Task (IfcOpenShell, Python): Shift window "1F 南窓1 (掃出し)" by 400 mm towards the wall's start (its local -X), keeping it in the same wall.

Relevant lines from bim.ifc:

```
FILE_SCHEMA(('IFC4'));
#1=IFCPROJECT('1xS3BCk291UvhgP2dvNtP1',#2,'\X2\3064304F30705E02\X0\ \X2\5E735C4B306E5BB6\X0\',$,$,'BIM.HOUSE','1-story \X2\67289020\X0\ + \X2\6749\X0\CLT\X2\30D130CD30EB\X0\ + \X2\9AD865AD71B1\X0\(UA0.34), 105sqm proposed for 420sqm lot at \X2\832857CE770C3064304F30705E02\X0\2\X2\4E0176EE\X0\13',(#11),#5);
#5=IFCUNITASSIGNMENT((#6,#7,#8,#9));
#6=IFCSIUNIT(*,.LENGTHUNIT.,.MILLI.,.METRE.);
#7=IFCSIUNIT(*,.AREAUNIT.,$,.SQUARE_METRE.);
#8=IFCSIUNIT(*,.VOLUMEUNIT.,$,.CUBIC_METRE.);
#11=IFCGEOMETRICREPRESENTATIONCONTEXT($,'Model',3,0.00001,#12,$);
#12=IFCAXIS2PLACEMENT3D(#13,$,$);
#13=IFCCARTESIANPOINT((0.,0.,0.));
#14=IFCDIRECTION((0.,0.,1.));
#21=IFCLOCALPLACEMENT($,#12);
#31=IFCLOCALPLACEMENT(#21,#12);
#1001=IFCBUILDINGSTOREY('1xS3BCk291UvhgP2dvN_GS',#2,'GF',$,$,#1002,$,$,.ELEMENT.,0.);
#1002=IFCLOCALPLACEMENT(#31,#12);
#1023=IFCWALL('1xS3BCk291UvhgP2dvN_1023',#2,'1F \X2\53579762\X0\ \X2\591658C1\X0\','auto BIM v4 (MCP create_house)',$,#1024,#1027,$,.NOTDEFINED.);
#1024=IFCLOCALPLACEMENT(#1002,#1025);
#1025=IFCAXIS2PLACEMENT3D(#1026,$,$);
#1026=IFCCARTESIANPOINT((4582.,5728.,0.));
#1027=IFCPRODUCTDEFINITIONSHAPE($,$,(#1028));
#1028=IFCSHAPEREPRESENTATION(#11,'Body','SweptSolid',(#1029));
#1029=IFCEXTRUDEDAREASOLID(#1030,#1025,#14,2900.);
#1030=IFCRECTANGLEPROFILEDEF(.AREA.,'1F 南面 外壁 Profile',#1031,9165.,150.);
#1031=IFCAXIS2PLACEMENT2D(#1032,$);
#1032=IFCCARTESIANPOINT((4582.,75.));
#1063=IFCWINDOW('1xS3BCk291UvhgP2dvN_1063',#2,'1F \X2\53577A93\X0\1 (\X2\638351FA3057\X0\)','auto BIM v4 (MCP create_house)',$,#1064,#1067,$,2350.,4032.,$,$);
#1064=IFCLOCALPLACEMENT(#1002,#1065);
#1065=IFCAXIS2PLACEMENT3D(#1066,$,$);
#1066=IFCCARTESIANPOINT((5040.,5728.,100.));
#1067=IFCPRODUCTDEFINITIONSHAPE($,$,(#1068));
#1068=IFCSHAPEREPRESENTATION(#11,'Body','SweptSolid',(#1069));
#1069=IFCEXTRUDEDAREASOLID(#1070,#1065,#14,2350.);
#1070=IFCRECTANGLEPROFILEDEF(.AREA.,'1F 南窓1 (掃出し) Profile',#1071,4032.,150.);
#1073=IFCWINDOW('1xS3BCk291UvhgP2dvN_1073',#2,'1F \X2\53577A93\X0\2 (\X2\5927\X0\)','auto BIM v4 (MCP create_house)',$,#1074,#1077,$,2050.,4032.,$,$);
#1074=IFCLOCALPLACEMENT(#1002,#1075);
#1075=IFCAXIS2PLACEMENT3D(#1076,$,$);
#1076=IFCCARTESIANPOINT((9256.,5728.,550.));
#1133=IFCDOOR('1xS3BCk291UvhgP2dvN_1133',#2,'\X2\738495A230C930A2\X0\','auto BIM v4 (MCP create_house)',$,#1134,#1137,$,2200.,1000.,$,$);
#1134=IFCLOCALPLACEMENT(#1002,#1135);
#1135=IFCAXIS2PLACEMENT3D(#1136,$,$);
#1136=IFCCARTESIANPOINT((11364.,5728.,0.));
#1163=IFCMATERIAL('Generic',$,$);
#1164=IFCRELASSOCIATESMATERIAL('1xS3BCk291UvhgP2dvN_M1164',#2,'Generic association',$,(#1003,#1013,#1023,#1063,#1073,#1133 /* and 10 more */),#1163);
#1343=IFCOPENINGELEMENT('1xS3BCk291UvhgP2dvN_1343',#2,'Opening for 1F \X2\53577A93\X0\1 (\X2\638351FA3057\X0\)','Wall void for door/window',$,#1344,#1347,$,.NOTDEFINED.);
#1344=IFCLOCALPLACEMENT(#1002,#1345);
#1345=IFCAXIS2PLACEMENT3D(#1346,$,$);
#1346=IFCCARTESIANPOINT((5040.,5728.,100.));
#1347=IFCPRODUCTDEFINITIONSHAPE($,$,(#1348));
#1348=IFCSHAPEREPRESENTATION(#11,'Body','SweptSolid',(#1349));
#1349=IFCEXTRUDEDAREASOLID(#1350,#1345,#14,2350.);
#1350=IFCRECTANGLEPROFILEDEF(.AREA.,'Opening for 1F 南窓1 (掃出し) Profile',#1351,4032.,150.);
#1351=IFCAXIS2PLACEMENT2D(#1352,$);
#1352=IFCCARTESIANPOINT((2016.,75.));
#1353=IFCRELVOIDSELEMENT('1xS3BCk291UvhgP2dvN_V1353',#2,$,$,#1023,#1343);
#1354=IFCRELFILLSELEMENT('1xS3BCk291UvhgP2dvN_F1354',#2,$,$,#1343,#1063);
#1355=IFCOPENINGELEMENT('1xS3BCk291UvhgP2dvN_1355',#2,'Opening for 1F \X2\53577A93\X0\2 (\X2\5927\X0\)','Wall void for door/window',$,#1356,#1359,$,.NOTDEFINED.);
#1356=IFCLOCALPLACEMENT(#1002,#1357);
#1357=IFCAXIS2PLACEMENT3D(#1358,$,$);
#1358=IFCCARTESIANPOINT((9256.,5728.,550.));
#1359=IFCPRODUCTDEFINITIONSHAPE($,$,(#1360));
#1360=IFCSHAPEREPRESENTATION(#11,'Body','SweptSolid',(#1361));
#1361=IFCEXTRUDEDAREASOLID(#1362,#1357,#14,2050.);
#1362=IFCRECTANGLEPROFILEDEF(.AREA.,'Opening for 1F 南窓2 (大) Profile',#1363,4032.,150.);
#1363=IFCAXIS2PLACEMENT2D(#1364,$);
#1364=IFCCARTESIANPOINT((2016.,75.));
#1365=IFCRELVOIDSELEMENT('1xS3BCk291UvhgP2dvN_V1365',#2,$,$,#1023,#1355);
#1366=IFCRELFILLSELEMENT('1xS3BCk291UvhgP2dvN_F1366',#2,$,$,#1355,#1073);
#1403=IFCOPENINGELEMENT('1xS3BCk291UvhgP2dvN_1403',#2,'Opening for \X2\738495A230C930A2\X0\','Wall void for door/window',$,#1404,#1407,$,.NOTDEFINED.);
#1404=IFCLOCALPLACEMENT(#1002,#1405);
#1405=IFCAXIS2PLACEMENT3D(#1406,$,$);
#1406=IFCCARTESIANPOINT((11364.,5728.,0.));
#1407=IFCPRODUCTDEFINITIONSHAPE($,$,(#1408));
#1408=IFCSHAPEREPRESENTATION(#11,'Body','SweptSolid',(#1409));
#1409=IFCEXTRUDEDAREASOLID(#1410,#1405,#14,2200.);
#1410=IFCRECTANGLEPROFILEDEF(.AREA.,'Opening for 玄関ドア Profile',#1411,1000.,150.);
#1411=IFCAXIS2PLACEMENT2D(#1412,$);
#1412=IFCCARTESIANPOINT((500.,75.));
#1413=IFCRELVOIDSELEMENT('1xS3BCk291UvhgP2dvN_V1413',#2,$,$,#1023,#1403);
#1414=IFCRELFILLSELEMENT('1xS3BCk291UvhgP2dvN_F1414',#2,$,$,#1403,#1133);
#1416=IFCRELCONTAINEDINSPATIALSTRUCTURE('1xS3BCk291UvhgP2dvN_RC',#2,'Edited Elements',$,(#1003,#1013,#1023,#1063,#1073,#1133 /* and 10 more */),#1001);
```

```python
import ifcopenshell
import ifcopenshell.api.geometry
import ifcopenshell.util.placement

model = ifcopenshell.open("bim.ifc")

window = model.by_guid("1xS3BCk291UvhgP2dvN_1063")
opening = window.FillsVoids[0].RelatingOpeningElement
wall = opening.VoidsElements[0].RelatingBuildingElement

wall_matrix = ifcopenshell.util.placement.get_local_placement(wall.ObjectPlacement)
shift = wall_matrix[:3, 0] * -400.0
before = ifcopenshell.util.placement.get_local_placement(window.ObjectPlacement)[:3, 3].copy()

# The window is not placed relative to its opening, so move both.
for product in (opening, window):
    matrix = ifcopenshell.util.placement.get_local_placement(product.ObjectPlacement)
    matrix[:3, 3] += shift
    ifcopenshell.api.geometry.edit_object_placement(model, product=product, matrix=matrix, is_si=False)

after = ifcopenshell.util.placement.get_local_placement(window.ObjectPlacement)[:3, 3]
print("window moved by", (after - before).round(3) + 0.0)

model.write("bim_v2.ifc")
```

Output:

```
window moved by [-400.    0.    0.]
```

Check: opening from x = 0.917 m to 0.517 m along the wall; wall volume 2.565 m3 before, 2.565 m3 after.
